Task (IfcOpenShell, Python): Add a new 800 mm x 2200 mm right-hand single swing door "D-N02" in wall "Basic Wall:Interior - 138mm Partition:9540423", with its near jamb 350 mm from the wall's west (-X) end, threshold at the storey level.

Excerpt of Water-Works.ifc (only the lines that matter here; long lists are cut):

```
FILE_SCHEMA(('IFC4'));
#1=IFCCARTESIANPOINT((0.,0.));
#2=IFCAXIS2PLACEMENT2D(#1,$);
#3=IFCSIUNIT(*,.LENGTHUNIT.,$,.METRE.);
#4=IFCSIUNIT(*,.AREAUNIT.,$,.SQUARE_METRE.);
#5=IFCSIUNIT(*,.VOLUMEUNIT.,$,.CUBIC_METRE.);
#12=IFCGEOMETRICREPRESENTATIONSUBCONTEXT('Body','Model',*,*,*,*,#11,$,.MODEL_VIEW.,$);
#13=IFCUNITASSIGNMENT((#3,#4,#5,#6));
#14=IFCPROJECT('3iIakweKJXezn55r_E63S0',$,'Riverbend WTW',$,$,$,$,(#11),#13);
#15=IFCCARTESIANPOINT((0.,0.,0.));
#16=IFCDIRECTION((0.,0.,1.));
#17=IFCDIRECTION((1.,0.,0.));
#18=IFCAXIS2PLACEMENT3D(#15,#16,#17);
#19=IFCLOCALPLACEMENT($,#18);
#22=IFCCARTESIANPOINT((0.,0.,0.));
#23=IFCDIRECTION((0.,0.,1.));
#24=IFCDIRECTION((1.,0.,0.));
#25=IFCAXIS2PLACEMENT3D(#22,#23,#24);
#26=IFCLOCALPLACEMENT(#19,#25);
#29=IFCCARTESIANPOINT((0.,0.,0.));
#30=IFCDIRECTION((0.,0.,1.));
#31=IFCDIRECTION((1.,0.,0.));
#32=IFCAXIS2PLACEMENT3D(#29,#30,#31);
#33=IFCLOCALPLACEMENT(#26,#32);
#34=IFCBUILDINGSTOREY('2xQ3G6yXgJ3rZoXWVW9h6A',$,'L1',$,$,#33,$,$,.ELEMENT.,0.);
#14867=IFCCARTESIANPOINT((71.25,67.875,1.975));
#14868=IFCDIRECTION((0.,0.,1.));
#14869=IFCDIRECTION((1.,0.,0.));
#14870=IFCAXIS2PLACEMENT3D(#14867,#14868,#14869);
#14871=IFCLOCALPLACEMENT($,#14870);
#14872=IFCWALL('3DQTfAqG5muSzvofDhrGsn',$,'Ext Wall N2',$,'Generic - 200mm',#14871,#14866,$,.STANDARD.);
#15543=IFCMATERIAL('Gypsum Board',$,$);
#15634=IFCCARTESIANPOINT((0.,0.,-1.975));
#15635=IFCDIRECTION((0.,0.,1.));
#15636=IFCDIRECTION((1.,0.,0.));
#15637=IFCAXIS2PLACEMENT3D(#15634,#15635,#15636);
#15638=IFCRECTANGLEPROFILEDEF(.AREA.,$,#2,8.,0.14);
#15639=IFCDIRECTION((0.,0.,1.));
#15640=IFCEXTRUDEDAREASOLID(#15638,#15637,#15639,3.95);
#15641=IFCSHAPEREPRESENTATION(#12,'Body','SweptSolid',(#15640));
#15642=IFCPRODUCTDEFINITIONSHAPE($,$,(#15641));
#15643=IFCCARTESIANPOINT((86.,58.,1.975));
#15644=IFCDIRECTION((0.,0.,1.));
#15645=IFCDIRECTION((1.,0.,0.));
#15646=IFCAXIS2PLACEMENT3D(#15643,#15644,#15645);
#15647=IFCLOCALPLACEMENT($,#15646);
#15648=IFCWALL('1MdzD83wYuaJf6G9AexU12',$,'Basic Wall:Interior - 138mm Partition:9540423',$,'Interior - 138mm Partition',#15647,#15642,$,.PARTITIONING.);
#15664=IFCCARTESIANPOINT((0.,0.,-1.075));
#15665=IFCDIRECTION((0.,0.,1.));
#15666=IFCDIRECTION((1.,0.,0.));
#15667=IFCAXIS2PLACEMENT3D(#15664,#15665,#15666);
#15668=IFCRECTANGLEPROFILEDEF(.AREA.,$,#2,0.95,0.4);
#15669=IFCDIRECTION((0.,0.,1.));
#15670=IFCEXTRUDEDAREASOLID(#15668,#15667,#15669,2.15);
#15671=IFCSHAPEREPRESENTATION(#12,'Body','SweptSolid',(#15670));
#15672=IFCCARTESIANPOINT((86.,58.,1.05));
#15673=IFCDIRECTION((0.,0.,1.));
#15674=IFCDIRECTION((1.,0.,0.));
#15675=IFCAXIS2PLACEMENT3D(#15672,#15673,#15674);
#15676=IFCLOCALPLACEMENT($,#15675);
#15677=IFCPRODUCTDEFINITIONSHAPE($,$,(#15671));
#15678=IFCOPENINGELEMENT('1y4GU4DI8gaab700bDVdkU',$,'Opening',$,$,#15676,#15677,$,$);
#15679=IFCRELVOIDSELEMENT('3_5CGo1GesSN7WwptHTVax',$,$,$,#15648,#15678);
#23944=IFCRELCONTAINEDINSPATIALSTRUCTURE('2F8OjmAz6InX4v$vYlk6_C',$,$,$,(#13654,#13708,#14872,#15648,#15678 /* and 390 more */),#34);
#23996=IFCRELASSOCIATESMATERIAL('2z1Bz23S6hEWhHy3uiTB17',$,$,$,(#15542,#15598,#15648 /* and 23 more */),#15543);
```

```python
import numpy as np
import ifcopenshell
import ifcopenshell.api.feature
import ifcopenshell.api.geometry
import ifcopenshell.api.root
import ifcopenshell.api.spatial
import ifcopenshell.geom
import ifcopenshell.util.element
import ifcopenshell.util.placement
import ifcopenshell.util.representation
import ifcopenshell.util.shape
import ifcopenshell.util.unit

model = ifcopenshell.open("Water-Works.ifc")
unit_scale = ifcopenshell.util.unit.calculate_unit_scale(model)
settings = ifcopenshell.geom.settings()


def volume(element):
    """Net volume in cubic metres, openings subtracted."""
    shape = ifcopenshell.geom.create_shape(settings, element)
    return ifcopenshell.util.shape.get_volume(shape.geometry)


wall = model.by_guid("1MdzD83wYuaJf6G9AexU12")
storey = ifcopenshell.util.element.get_container(wall, ifc_class="IfcBuildingStorey")
context = ifcopenshell.util.representation.get_context(model, "Model", "Body", "MODEL_VIEW")
before = volume(wall)

width, height, from_end, sill = 0.8, 2.2, 0.35, 0.0  # metres

# The wall runs along its own X axis, and the end named is its -X end.
wall_shape = ifcopenshell.geom.create_shape(settings, wall)
x, y, z = ifcopenshell.util.shape.get_vertices(wall_shape.geometry).T
start = x.min() + from_end
face, thickness = float(y.min()), float(y.max() - y.min())
wall_matrix = ifcopenshell.util.placement.get_local_placement(wall.ObjectPlacement)
level = ifcopenshell.util.placement.get_local_placement(storey.ObjectPlacement)[2, 3]


def in_wall(x, y):
    """Placement at x, y metres in the wall's axes, at sill height."""
    matrix = wall_matrix.copy()
    matrix[:, 3] = wall_matrix @ np.array([x / unit_scale, y / unit_scale, 0.0, 1.0])
    matrix[2, 3] = level + sill / unit_scale
    return matrix


# Opening: a box that overshoots both wall faces by 50 mm.
opening = ifcopenshell.api.root.create_entity(model, ifc_class="IfcOpeningElement", predefined_type="OPENING")
box = ifcopenshell.api.geometry.add_wall_representation(
    model, context=context, length=width, height=height, thickness=thickness + 0.1
)
ifcopenshell.api.geometry.assign_representation(model, product=opening, representation=box)
ifcopenshell.api.geometry.edit_object_placement(model, product=opening, matrix=in_wall(start, face - 0.05), is_si=False)
ifcopenshell.api.feature.add_feature(model, feature=opening, element=wall)

door = ifcopenshell.api.root.create_entity(model, ifc_class="IfcDoor", name="D-N02", predefined_type="DOOR")
door.OverallWidth, door.OverallHeight = width / unit_scale, height / unit_scale
door.OperationType = "SINGLE_SWING_RIGHT"
body = ifcopenshell.api.geometry.add_door_representation(
    model,
    context=context,
    overall_width=door.OverallWidth,
    overall_height=door.OverallHeight,
    operation_type="SINGLE_SWING_RIGHT",
    lining_properties={"LiningDepth": thickness / unit_scale, "ThresholdDepth": thickness / unit_scale},
)
ifcopenshell.api.geometry.assign_representation(model, product=door, representation=body)
ifcopenshell.api.spatial.assign_container(model, products=[door], relating_structure=storey)
ifcopenshell.api.feature.add_filling(model, opening=opening, element=door)

# The lining spans the wall, so the door starts at the wall face.
ifcopenshell.api.geometry.edit_object_placement(model, product=door, matrix=in_wall(start, face), is_si=False)

after = volume(wall)

print(f"wall volume {before:.3f} -> {after:.3f} m3")

model.write("Water-Works_rev.ifc")
```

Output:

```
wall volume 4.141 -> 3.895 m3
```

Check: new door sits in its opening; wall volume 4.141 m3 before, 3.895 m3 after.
